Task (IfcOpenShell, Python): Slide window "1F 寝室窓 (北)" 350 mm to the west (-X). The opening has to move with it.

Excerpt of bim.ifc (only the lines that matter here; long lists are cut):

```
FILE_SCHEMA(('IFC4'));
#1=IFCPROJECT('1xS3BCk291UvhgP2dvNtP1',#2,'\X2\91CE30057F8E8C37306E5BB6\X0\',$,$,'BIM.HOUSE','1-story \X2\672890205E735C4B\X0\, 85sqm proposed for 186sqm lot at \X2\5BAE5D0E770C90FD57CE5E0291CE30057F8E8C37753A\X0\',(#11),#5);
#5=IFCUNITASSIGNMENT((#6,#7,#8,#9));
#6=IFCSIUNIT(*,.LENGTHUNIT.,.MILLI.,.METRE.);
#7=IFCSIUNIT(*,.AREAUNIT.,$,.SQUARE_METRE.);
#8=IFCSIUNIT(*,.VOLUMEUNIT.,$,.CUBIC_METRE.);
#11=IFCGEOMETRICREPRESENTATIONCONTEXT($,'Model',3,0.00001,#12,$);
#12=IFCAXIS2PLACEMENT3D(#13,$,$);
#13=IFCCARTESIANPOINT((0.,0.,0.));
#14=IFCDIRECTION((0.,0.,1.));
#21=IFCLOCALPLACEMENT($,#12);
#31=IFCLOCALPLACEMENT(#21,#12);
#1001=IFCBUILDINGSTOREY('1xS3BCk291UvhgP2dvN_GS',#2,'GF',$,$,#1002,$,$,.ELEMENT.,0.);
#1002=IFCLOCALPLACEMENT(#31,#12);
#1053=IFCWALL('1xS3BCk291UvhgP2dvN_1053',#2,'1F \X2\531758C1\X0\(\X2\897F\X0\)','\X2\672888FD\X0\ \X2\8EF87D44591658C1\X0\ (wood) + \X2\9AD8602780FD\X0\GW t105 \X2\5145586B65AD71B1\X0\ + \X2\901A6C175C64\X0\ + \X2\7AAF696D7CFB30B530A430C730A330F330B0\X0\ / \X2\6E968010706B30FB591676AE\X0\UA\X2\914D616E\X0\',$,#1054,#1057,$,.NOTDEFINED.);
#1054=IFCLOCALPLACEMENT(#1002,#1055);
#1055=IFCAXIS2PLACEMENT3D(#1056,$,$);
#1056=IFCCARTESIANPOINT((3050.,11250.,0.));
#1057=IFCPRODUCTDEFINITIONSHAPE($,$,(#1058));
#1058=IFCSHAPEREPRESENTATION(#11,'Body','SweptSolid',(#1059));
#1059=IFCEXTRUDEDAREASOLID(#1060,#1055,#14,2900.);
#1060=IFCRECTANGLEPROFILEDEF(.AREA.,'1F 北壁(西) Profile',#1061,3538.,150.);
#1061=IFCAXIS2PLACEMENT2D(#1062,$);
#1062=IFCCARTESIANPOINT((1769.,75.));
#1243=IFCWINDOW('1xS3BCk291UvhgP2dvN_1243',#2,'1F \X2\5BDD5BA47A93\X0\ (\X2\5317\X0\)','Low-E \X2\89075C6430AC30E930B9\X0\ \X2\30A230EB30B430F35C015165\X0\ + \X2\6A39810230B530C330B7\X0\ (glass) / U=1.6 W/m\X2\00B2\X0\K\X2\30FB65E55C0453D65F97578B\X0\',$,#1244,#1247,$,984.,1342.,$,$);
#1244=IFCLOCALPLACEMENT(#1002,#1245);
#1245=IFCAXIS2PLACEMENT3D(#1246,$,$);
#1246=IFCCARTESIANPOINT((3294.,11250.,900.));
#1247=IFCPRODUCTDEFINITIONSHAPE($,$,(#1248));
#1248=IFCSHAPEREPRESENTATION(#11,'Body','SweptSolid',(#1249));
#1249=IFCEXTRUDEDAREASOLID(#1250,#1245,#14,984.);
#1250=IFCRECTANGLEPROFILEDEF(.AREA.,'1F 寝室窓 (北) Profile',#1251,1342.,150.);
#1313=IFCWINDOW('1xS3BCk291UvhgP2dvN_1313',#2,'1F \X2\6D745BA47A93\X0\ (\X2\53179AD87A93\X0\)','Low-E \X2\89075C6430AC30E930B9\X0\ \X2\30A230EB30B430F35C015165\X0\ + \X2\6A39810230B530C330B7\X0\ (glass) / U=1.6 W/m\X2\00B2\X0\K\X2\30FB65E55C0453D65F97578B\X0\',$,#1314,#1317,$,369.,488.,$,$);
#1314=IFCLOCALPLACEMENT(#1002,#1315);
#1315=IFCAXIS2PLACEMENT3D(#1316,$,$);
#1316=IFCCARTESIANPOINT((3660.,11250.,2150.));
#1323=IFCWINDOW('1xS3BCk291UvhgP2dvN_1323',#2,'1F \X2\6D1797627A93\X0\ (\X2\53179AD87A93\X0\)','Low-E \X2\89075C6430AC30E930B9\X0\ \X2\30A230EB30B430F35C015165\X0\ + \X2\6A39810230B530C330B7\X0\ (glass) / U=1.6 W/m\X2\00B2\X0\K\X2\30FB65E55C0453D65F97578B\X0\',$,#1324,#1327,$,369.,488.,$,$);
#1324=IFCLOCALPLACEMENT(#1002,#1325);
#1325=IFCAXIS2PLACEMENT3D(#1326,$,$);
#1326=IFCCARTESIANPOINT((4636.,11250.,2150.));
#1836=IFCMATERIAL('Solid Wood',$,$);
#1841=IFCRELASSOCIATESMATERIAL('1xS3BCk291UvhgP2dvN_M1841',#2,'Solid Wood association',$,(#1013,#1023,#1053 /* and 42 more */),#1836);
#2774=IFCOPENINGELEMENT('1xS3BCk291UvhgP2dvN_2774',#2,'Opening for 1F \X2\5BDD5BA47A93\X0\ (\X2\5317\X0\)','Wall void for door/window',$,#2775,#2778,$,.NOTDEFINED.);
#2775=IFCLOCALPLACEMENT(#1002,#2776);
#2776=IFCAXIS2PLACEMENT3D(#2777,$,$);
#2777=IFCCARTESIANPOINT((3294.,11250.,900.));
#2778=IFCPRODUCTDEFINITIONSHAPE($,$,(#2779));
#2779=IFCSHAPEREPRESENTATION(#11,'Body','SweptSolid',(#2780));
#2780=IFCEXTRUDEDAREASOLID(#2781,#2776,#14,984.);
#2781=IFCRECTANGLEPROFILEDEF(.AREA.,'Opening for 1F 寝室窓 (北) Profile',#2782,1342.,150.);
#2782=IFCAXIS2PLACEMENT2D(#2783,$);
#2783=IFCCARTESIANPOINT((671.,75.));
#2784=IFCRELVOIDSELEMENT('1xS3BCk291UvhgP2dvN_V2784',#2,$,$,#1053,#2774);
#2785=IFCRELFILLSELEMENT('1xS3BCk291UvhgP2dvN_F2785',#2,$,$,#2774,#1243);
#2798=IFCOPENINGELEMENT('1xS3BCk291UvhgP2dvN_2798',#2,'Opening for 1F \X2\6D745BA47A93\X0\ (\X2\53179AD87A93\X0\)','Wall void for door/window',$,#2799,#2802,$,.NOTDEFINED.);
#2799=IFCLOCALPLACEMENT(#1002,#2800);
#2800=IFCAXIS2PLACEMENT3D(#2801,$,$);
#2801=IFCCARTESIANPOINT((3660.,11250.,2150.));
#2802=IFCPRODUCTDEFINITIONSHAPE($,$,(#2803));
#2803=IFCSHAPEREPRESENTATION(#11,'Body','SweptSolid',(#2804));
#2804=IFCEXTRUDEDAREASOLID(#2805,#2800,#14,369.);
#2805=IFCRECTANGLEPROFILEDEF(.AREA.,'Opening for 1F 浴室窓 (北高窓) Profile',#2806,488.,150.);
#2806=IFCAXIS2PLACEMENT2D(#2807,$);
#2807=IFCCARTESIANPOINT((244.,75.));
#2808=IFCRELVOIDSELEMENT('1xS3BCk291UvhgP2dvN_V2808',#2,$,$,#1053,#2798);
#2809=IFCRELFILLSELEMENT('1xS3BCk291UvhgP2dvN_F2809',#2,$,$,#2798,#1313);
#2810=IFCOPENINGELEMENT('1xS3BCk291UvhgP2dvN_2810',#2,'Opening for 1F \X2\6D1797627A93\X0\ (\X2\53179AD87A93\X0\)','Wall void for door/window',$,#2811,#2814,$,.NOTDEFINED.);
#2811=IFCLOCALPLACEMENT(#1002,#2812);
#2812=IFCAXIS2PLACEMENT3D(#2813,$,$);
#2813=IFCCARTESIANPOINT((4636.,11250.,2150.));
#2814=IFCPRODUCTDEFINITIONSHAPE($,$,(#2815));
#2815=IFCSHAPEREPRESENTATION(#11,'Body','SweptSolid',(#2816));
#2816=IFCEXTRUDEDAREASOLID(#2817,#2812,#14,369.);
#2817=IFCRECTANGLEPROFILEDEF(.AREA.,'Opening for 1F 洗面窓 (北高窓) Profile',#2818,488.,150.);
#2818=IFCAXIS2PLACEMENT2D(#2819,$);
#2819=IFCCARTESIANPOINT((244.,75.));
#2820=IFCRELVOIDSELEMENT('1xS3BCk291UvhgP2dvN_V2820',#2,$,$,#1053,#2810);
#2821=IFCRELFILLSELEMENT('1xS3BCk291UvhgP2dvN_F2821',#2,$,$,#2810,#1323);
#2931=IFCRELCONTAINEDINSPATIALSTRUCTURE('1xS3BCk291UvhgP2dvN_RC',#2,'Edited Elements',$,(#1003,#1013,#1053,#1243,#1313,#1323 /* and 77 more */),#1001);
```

```python
import ifcopenshell
import ifcopenshell.api.geometry
import ifcopenshell.util.placement
import ifcopenshell.util.unit

model = ifcopenshell.open("bim.ifc")
unit_scale = ifcopenshell.util.unit.calculate_unit_scale(model)

window = model.by_id(1243)
opening = window.FillsVoids[0].RelatingOpeningElement
wall = opening.VoidsElements[0].RelatingBuildingElement

wall_matrix = ifcopenshell.util.placement.get_local_placement(wall.ObjectPlacement)
shift = wall_matrix[:3, 0] * -0.35 / unit_scale
before = ifcopenshell.util.placement.get_local_placement(window.ObjectPlacement)[:3, 3].copy()

# The window is not placed relative to its opening, so move both.
for product in (opening, window):
    matrix = ifcopenshell.util.placement.get_local_placement(product.ObjectPlacement)
    matrix[:3, 3] += shift
    ifcopenshell.api.geometry.edit_object_placement(model, product=product, matrix=matrix, is_si=False)

after = ifcopenshell.util.placement.get_local_placement(window.ObjectPlacement)[:3, 3]
print("window moved by", (after - before).round(3) + 0.0)

model.write("bim_rev.ifc")
```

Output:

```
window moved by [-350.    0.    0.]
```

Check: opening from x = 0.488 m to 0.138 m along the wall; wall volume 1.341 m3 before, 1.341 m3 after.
